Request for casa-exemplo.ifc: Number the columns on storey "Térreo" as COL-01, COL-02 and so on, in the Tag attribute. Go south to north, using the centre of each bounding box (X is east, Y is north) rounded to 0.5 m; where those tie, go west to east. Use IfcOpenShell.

First a look at what the model holds.

```python
import ifcopenshell
import ifcopenshell.util.element
import ifcopenshell.util.placement

model = ifcopenshell.open("casa-exemplo.ifc")
print(model.schema)
storey = next(s for s in model.by_type("IfcBuildingStorey") if s.Name == "Térreo")
columns = [e for e in ifcopenshell.util.element.get_decomposition(storey) if e.is_a("IfcColumn")]
for e in sorted(columns, key=lambda e: e.id()):
    origin = ifcopenshell.util.placement.get_local_placement(e.ObjectPlacement)[:3, 3]
    print(e.id(), e.Tag, e.Name, origin.round(2) + 0.0, sep=" | ")
```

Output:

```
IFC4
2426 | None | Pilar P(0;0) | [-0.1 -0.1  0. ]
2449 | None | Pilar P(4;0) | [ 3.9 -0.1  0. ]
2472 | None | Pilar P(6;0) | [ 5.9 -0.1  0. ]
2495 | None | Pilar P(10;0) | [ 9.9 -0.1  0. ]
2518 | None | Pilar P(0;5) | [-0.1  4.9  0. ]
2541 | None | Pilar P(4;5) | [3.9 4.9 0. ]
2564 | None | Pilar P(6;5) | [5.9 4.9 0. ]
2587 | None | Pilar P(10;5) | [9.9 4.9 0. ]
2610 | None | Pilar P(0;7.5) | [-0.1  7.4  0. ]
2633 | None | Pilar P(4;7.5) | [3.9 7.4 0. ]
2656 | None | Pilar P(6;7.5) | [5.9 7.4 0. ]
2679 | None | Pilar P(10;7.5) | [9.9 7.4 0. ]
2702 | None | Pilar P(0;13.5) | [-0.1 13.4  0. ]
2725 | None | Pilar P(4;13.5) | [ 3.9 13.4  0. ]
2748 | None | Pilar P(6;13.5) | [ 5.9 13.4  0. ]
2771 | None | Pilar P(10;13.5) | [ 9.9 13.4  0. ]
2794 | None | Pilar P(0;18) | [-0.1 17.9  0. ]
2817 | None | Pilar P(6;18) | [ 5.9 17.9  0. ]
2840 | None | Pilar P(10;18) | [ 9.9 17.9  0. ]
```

```python
import ifcopenshell
import ifcopenshell.geom
import ifcopenshell.util.element
import ifcopenshell.util.shape

model = ifcopenshell.open("casa-exemplo.ifc")
settings = ifcopenshell.geom.settings()
settings.set("use-world-coords", True)


def centre(element):
    shape = ifcopenshell.geom.create_shape(settings, element)
    return ifcopenshell.util.shape.get_bbox_centroid(shape.geometry)


storey = next(s for s in model.by_type("IfcBuildingStorey") if s.Name == "Térreo")
columns = [e for e in ifcopenshell.util.element.get_decomposition(storey) if e.is_a("IfcColumn")]

# Insertion points can sit at a corner or the storey origin, so sort by the geometry (in metres).
centres = {e: centre(e) for e in columns}
columns.sort(key=lambda e: (round(centres[e][1] / 0.5), centres[e][0]))

for i, e in enumerate(columns, start=1):
    number = f"COL-{i:02d}"
    e.Tag = number
    print(e.id(), number)

model.write("casa-exemplo-out.ifc")
```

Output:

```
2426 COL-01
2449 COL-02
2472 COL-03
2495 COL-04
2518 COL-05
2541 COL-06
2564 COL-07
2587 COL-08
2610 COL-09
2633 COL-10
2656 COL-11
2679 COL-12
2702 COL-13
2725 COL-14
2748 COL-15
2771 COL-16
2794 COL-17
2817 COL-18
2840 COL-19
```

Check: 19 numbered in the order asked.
